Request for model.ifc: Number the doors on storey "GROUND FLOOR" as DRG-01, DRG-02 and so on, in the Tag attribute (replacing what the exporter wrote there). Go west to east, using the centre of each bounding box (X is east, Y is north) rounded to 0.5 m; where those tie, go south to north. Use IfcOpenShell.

First a look at what the model holds.

```python
import ifcopenshell
import ifcopenshell.util.element
import ifcopenshell.util.placement

model = ifcopenshell.open("model.ifc")
print(model.schema)
storey = next(s for s in model.by_type("IfcBuildingStorey") if s.Name == "GROUND FLOOR")
doors = [e for e in ifcopenshell.util.element.get_decomposition(storey) if e.is_a("IfcDoor")]
for e in sorted(doors, key=lambda e: e.id()):
    origin = ifcopenshell.util.placement.get_local_placement(e.ObjectPlacement)[:3, 3]
    print(e.id(), e.Tag, e.Name, origin.round(2) + 0.0, sep=" | ")
```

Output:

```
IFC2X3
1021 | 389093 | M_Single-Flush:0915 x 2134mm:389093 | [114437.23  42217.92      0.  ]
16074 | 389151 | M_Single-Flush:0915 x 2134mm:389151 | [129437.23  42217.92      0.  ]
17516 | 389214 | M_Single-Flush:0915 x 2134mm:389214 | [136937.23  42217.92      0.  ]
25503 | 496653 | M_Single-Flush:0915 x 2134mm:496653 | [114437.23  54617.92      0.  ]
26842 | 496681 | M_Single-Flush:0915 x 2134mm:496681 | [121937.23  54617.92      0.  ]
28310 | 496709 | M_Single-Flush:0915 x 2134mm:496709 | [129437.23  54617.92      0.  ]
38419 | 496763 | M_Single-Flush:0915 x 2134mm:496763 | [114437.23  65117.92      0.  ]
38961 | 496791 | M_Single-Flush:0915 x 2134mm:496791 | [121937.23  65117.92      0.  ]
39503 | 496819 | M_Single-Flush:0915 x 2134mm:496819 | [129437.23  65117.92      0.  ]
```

```python
import ifcopenshell
import ifcopenshell.geom
import ifcopenshell.util.element
import ifcopenshell.util.shape

model = ifcopenshell.open("model.ifc")
settings = ifcopenshell.geom.settings()
settings.set("use-world-coords", True)


def centre(element):
    shape = ifcopenshell.geom.create_shape(settings, element)
    return ifcopenshell.util.shape.get_bbox_centroid(shape.geometry)


storey = next(s for s in model.by_type("IfcBuildingStorey") if s.Name == "GROUND FLOOR")
doors = [e for e in ifcopenshell.util.element.get_decomposition(storey) if e.is_a("IfcDoor")]

# Insertion points can sit at a corner or the storey origin, so sort by the geometry (in metres).
centres = {e: centre(e) for e in doors}
doors.sort(key=lambda e: (round(centres[e][0] / 0.5), centres[e][1]))

for i, e in enumerate(doors, start=1):
    number = f"DRG-{i:02d}"
    e.Tag = number
    print(e.id(), number)

model.write("model-out.ifc")
```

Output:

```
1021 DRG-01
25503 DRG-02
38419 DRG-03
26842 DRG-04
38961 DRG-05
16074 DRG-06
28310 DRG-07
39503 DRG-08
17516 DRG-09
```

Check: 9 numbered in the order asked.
